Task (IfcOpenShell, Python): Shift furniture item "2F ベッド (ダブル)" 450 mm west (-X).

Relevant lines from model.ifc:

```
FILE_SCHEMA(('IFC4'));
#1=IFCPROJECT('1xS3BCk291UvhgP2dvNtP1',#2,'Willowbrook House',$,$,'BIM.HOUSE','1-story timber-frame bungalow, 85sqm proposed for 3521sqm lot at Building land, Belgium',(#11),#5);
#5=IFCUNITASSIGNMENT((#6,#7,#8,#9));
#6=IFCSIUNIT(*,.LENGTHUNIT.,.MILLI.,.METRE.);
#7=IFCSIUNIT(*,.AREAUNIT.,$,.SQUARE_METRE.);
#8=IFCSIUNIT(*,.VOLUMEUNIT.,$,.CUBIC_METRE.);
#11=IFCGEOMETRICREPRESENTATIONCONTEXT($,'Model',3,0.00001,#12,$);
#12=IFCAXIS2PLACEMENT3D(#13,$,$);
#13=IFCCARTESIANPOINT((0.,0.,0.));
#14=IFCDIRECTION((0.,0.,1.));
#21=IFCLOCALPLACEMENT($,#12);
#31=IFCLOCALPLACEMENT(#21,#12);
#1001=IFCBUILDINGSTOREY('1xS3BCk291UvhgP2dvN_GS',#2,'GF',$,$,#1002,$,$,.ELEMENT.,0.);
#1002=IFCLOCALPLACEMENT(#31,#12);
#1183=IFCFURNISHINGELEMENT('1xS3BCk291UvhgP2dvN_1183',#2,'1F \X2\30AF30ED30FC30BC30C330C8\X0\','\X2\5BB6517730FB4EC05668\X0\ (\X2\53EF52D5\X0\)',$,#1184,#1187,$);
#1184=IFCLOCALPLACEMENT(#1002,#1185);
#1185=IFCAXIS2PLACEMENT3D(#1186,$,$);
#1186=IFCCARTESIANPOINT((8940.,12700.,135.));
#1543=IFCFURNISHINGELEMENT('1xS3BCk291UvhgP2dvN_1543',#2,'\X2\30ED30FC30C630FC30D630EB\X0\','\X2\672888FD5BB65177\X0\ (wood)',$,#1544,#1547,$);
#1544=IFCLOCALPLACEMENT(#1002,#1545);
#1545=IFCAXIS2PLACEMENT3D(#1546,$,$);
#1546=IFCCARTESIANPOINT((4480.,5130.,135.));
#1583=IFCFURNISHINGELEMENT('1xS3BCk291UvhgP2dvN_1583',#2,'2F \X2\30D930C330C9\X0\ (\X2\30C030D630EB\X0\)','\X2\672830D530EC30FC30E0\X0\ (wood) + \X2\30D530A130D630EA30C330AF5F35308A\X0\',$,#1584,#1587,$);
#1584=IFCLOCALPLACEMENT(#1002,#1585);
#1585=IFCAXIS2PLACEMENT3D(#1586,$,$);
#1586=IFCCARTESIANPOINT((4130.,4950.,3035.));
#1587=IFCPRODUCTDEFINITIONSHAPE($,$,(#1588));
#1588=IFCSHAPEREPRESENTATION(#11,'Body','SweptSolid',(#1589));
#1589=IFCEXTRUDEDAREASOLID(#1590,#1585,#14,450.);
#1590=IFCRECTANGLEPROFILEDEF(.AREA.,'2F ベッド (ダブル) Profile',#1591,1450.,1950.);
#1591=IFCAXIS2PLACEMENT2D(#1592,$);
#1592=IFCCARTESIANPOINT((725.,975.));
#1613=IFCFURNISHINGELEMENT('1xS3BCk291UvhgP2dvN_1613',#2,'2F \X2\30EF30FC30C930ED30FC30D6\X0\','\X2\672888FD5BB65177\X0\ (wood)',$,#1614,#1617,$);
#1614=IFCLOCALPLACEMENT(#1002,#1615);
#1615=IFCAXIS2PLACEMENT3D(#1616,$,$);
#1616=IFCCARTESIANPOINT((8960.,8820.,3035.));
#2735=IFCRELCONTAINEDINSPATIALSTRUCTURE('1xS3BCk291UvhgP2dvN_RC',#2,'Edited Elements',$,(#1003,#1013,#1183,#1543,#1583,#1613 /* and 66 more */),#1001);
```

```python
import ifcopenshell
import ifcopenshell.api.geometry
import ifcopenshell.util.placement
import ifcopenshell.util.unit

model = ifcopenshell.open("model.ifc")
unit_scale = ifcopenshell.util.unit.calculate_unit_scale(model)

item = model.by_guid("1xS3BCk291UvhgP2dvN_1583")
matrix = ifcopenshell.util.placement.get_local_placement(item.ObjectPlacement)
matrix[0, 3] -= 0.45 / unit_scale
ifcopenshell.api.geometry.edit_object_placement(model, product=item, matrix=matrix, is_si=False)

print(ifcopenshell.util.placement.get_local_placement(item.ObjectPlacement).round(3) + 0.0)

model.write("model_edited.ifc")
```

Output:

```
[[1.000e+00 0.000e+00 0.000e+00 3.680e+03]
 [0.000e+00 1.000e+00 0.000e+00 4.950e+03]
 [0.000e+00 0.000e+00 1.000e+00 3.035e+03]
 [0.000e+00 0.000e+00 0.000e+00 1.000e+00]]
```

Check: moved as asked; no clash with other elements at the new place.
